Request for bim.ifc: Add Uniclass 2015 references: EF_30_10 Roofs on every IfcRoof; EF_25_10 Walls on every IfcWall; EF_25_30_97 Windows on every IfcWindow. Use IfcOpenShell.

First a look at what the model holds.

```python
import ifcopenshell

model = ifcopenshell.open("bim.ifc")
print(model.schema)
print("classifications:", [c.Name for c in model.by_type("IfcClassification")])
for ifc_class in ("IfcDoor", "IfcRoof", "IfcStair", "IfcWall", "IfcWindow"):
    print(ifc_class, len(model.by_type(ifc_class)))
```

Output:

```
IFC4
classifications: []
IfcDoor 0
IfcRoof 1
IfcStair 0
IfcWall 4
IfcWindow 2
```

```python
import ifcopenshell
import ifcopenshell.api.classification

model = ifcopenshell.open("bim.ifc")

system = ifcopenshell.api.classification.add_classification(model, classification="Uniclass 2015")

codes = {
    "IfcRoof": ("EF_30_10", "Roofs"),
    "IfcWall": ("EF_25_10", "Walls"),
    "IfcWindow": ("EF_25_30_97", "Windows"),
}
for ifc_class, (code, name) in codes.items():
    products = model.by_type(ifc_class)
    ifcopenshell.api.classification.add_reference(
        model, products=products, classification=system, identification=code, name=name
    )
    print(code, len(products))

model.write("bim-out.ifc")
```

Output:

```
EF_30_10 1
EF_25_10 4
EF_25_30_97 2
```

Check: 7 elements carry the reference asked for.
